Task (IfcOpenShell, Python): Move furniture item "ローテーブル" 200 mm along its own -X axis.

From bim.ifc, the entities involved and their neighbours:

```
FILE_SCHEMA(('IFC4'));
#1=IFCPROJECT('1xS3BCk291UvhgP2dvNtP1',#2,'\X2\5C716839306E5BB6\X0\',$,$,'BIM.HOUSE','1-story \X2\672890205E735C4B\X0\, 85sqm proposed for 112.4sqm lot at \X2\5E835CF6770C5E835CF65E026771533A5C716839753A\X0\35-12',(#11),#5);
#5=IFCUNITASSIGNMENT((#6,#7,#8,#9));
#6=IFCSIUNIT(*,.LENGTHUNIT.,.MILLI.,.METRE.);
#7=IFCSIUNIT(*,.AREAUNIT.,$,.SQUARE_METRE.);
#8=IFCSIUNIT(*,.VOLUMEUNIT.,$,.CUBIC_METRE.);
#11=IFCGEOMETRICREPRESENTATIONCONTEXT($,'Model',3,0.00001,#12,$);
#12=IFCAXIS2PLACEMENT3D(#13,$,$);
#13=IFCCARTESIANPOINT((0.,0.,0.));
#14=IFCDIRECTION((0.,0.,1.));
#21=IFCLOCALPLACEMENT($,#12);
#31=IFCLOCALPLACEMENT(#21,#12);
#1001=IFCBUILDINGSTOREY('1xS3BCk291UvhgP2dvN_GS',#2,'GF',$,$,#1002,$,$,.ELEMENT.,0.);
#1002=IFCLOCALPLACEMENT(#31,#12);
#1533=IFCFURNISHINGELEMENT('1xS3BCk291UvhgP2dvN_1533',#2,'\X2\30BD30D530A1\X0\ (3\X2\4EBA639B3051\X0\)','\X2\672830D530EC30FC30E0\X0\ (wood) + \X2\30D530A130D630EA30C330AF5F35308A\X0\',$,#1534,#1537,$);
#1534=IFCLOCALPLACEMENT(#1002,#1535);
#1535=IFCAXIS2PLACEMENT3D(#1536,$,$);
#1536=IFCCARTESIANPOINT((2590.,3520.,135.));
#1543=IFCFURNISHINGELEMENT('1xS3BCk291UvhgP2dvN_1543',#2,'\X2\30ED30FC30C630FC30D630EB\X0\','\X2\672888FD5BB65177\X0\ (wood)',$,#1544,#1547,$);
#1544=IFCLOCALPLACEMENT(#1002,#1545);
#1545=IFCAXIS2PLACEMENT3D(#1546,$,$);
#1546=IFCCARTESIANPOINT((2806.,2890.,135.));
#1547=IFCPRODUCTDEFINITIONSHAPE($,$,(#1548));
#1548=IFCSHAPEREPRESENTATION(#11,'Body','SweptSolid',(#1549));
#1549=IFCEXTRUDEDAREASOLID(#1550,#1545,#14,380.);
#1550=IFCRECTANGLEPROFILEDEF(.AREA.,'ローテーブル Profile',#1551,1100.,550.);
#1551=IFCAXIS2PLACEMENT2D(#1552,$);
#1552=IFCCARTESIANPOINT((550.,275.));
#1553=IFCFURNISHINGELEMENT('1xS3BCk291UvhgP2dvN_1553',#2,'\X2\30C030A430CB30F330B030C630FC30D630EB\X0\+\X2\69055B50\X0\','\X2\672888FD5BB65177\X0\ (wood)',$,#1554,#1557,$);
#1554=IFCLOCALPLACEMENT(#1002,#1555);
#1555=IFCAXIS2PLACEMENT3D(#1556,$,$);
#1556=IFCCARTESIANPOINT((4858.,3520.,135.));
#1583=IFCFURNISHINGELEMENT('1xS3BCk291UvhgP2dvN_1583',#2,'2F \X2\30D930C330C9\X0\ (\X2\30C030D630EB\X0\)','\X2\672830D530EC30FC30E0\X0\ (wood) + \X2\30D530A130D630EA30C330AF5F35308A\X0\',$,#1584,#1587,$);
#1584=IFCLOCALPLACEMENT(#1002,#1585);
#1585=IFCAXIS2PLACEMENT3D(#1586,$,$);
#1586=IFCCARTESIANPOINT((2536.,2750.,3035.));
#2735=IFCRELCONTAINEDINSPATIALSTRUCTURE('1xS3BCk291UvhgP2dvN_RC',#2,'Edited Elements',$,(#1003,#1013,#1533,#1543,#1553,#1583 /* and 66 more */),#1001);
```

```python
import ifcopenshell
import ifcopenshell.api.geometry
import ifcopenshell.util.placement
import ifcopenshell.util.unit

model = ifcopenshell.open("bim.ifc")
unit_scale = ifcopenshell.util.unit.calculate_unit_scale(model)

item = model.by_id(1543)
matrix = ifcopenshell.util.placement.get_local_placement(item.ObjectPlacement)
matrix[:3, 3] -= matrix[:3, 0] * 0.2 / unit_scale
ifcopenshell.api.geometry.edit_object_placement(model, product=item, matrix=matrix, is_si=False)

print(ifcopenshell.util.placement.get_local_placement(item.ObjectPlacement).round(3) + 0.0)

model.write("bim_updated.ifc")
```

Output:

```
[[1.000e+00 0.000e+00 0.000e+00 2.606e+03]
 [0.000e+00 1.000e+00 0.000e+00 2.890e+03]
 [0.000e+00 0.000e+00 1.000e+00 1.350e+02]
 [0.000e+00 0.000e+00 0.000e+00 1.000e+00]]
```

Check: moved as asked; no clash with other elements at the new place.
